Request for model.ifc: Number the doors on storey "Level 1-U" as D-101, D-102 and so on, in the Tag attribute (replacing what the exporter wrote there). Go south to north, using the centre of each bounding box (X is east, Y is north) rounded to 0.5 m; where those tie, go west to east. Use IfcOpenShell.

First a look at what the model holds.

```python
import ifcopenshell
import ifcopenshell.util.element
import ifcopenshell.util.placement

model = ifcopenshell.open("model.ifc")
print(model.schema)
storey = next(s for s in model.by_type("IfcBuildingStorey") if s.Name == "Level 1-U")
doors = [e for e in ifcopenshell.util.element.get_decomposition(storey) if e.is_a("IfcDoor")]
for e in sorted(doors, key=lambda e: e.id()):
    origin = ifcopenshell.util.placement.get_local_placement(e.ObjectPlacement)[:3, 3]
    print(e.id(), e.Tag, e.Name, origin.round(2) + 0.0, sep=" | ")
```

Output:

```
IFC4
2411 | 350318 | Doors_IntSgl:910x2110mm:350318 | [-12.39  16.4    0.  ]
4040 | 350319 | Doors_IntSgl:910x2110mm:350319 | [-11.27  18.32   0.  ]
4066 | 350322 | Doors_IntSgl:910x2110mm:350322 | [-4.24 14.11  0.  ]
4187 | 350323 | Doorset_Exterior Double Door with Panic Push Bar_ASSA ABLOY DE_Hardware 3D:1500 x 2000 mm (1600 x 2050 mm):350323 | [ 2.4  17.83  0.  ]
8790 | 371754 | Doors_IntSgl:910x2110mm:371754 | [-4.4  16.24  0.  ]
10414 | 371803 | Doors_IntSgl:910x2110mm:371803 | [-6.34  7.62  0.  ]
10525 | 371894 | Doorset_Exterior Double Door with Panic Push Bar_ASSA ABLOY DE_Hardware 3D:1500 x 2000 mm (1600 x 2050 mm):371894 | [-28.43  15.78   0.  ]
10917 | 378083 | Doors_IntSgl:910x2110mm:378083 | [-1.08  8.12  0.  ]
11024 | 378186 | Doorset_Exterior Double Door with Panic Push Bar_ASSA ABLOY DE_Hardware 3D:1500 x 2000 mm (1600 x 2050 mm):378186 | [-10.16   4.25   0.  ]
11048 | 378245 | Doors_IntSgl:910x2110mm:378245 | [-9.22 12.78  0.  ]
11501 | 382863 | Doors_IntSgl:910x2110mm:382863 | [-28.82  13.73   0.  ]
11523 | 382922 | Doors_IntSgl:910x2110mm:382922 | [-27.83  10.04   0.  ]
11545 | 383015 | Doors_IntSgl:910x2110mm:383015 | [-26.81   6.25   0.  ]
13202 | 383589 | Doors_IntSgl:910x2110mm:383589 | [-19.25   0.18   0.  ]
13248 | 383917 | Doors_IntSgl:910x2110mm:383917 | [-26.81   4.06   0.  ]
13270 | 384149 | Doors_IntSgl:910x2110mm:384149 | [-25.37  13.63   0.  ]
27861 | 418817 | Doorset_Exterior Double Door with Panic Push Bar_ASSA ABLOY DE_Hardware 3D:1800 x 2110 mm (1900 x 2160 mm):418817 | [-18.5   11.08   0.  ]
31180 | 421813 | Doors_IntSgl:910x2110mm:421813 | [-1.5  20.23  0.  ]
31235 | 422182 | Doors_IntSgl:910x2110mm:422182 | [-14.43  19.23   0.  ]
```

```python
import ifcopenshell
import ifcopenshell.geom
import ifcopenshell.util.element
import ifcopenshell.util.shape

model = ifcopenshell.open("model.ifc")
settings = ifcopenshell.geom.settings()
settings.set("use-world-coords", True)


def centre(element):
    shape = ifcopenshell.geom.create_shape(settings, element)
    return ifcopenshell.util.shape.get_bbox_centroid(shape.geometry)


storey = next(s for s in model.by_type("IfcBuildingStorey") if s.Name == "Level 1-U")
doors = [e for e in ifcopenshell.util.element.get_decomposition(storey) if e.is_a("IfcDoor")]

# Insertion points can sit at a corner or the storey origin, so sort by the geometry (in metres).
centres = {e: centre(e) for e in doors}
doors.sort(key=lambda e: (round(centres[e][1] / 0.5), centres[e][0]))

for i, e in enumerate(doors, start=1):
    number = f"D-1{i:02d}"
    e.Tag = number
    print(e.id(), number)

model.write("model_v2.ifc")
```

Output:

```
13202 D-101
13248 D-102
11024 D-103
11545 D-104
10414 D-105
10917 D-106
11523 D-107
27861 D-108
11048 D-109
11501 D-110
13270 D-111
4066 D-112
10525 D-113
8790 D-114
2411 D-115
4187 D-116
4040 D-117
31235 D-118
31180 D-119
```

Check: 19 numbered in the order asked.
